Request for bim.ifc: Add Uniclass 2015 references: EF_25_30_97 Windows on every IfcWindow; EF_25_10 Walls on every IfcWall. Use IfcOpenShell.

First a look at what the model holds.

```python
import ifcopenshell

model = ifcopenshell.open("bim.ifc")
print(model.schema)
print("classifications:", [c.Name for c in model.by_type("IfcClassification")])
for ifc_class in ("IfcDoor", "IfcRoof", "IfcStair", "IfcWall", "IfcWindow"):
    print(ifc_class, len(model.by_type(ifc_class)))
```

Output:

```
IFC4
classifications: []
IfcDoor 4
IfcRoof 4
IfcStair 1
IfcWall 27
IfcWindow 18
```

```python
import ifcopenshell
import ifcopenshell.api.classification

model = ifcopenshell.open("bim.ifc")

system = ifcopenshell.api.classification.add_classification(model, classification="Uniclass 2015")

codes = {
    "IfcWindow": ("EF_25_30_97", "Windows"),
    "IfcWall": ("EF_25_10", "Walls"),
}
for ifc_class, (code, name) in codes.items():
    products = model.by_type(ifc_class)
    ifcopenshell.api.classification.add_reference(
        model, products=products, classification=system, identification=code, name=name
    )
    print(code, len(products))

model.write("bim-out.ifc")
```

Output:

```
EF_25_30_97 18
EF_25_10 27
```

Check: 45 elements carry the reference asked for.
